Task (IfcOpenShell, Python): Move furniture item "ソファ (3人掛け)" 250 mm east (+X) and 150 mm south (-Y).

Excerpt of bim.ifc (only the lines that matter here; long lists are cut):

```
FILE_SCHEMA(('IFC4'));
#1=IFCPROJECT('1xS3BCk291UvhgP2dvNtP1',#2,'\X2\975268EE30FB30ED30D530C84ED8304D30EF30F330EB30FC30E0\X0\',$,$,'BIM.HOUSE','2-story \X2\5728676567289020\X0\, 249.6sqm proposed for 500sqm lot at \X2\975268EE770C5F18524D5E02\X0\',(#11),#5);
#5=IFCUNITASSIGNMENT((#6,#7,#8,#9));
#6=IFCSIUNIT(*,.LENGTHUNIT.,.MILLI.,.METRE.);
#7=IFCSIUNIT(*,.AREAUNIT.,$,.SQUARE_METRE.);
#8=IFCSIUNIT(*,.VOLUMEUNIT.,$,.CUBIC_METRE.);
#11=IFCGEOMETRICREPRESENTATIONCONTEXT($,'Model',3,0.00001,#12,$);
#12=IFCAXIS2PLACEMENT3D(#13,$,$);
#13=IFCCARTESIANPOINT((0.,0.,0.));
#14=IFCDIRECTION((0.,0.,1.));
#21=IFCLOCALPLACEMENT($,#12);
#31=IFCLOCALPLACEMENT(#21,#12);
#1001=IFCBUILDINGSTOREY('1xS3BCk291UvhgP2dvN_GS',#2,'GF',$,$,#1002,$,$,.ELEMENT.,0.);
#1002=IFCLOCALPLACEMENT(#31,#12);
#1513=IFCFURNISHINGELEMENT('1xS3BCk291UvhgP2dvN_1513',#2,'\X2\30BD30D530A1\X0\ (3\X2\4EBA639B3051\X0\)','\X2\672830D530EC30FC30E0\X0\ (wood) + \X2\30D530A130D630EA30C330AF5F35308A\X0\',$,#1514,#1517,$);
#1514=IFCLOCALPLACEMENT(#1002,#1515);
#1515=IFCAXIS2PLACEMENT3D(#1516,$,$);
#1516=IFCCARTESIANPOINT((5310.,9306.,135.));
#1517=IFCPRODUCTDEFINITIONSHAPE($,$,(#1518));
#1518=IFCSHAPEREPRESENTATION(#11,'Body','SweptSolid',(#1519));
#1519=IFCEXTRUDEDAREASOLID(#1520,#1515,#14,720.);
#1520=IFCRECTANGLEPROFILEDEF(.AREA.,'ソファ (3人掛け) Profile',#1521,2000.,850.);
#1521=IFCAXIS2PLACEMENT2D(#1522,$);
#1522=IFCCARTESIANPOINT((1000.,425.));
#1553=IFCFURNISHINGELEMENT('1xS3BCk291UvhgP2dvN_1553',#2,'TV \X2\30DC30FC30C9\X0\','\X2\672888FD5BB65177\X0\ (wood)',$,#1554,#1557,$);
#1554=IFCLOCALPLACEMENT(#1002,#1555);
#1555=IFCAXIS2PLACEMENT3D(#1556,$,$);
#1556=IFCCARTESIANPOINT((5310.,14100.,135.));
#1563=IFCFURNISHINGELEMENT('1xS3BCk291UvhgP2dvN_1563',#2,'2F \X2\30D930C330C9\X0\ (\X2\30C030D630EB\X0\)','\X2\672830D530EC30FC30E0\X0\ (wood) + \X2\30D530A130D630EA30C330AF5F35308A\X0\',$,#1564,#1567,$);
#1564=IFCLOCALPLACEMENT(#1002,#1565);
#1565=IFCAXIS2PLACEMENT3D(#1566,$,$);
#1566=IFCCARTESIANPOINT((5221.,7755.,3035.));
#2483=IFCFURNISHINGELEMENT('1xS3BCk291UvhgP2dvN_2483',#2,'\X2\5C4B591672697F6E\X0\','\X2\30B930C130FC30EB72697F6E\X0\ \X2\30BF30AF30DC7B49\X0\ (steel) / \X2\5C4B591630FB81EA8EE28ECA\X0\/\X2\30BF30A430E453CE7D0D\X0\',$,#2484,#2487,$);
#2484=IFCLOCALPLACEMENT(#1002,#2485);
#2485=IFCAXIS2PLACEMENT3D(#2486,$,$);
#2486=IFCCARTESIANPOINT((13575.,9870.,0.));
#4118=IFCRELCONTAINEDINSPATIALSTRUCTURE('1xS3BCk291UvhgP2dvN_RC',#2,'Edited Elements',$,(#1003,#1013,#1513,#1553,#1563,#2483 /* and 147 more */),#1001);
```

```python
import ifcopenshell
import ifcopenshell.api.geometry
import ifcopenshell.util.placement

model = ifcopenshell.open("bim.ifc")

item = model.by_guid("1xS3BCk291UvhgP2dvN_1513")
matrix = ifcopenshell.util.placement.get_local_placement(item.ObjectPlacement)
matrix[0, 3] += 250.0
matrix[1, 3] -= 150.0
ifcopenshell.api.geometry.edit_object_placement(model, product=item, matrix=matrix, is_si=False)

print(ifcopenshell.util.placement.get_local_placement(item.ObjectPlacement).round(3) + 0.0)

model.write("bim_edited.ifc")
```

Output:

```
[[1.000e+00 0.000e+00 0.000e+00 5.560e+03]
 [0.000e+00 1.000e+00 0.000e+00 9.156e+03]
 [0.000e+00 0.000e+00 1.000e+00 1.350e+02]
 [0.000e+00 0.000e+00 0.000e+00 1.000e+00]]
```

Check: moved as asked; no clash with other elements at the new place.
